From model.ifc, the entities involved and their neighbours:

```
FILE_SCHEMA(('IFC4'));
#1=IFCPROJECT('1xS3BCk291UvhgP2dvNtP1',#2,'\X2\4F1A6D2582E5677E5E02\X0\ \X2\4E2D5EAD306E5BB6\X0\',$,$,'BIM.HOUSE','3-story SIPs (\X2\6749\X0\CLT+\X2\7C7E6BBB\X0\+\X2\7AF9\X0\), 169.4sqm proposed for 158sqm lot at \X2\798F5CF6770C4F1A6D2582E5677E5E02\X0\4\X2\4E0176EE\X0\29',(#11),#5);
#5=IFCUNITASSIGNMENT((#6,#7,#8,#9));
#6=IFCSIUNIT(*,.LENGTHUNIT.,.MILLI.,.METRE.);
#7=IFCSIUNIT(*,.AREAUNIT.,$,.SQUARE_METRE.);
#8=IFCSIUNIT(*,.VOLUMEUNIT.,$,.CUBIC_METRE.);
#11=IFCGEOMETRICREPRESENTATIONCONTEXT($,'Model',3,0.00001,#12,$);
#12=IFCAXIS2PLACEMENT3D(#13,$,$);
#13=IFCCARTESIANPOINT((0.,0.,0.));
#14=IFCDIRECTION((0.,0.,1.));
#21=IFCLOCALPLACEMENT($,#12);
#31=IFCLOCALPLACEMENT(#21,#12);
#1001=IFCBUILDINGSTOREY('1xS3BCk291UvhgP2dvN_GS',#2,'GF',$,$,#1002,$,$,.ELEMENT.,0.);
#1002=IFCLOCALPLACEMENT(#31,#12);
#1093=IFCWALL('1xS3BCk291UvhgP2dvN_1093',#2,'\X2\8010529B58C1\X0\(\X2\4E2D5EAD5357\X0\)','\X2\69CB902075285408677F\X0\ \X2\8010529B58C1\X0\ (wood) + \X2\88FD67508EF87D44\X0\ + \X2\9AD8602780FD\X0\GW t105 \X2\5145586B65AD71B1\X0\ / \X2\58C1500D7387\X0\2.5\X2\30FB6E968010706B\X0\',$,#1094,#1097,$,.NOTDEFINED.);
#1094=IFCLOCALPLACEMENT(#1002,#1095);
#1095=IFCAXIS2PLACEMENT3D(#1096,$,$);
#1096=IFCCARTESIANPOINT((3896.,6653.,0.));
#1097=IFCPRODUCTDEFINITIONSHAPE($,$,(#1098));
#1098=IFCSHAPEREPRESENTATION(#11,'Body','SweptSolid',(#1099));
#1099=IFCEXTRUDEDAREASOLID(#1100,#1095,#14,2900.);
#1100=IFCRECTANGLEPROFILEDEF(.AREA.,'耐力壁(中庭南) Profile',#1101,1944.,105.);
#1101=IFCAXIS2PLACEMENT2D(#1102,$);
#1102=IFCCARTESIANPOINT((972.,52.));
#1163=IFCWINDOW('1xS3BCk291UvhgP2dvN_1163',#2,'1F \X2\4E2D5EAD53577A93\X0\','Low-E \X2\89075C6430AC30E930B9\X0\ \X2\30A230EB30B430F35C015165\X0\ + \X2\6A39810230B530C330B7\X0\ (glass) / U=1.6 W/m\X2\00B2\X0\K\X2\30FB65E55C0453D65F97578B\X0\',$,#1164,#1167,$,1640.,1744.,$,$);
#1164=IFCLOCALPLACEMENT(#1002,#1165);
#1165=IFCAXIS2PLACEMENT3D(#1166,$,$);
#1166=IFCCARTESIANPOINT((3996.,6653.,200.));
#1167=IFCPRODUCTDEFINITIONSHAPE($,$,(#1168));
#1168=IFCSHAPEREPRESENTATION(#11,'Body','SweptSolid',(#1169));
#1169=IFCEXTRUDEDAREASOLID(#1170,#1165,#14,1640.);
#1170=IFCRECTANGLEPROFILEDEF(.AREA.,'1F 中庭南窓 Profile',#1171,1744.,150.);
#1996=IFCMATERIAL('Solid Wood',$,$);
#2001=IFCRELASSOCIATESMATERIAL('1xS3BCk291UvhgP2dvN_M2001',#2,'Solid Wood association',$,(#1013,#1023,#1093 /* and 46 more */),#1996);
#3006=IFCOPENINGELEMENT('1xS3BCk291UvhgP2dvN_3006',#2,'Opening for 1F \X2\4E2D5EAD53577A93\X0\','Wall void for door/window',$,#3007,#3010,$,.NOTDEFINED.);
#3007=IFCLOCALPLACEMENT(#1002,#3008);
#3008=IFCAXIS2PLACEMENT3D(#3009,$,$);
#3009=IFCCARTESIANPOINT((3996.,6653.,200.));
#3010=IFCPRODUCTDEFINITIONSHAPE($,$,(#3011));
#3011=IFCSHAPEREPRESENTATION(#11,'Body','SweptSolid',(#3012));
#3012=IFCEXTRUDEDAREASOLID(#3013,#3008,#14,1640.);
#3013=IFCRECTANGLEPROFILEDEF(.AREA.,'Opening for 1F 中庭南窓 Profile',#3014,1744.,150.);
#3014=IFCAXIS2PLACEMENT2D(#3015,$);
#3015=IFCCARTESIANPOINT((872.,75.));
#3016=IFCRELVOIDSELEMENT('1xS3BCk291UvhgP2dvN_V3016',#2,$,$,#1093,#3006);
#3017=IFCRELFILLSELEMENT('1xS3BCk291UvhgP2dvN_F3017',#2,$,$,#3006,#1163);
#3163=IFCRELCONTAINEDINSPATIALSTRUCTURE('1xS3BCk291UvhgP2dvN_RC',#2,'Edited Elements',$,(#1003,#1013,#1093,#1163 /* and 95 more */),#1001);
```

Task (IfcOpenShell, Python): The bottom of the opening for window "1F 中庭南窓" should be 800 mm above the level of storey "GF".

```python
import numpy as np
import ifcopenshell
import ifcopenshell.api.geometry
import ifcopenshell.geom
import ifcopenshell.util.element
import ifcopenshell.util.placement
import ifcopenshell.util.shape
import ifcopenshell.util.unit

model = ifcopenshell.open("model.ifc")
unit_scale = ifcopenshell.util.unit.calculate_unit_scale(model)

window = model.by_id(1163)
opening = window.FillsVoids[0].RelatingOpeningElement
storey = ifcopenshell.util.element.get_container(window, ifc_class="IfcBuildingStorey")
level = ifcopenshell.util.placement.get_local_placement(storey.ObjectPlacement)[2, 3]

# The opening's origin need not be at the sill, so measure its lowest point.
shape = ifcopenshell.geom.create_shape(ifcopenshell.geom.settings(), opening)
bottom = ifcopenshell.util.shape.get_shape_bottom_elevation(shape, shape.geometry) / unit_scale
dz = level + 0.8 / unit_scale - bottom

shift = np.array([0.0, 0.0, dz])
# The window is not placed relative to its opening, so move both.
for product in (opening, window):
    matrix = ifcopenshell.util.placement.get_local_placement(product.ObjectPlacement)
    matrix[:3, 3] += shift
    ifcopenshell.api.geometry.edit_object_placement(model, product=product, matrix=matrix, is_si=False)

print(f"moved by {dz * unit_scale:+.3f} m")

model.write("model_updated.ifc")
```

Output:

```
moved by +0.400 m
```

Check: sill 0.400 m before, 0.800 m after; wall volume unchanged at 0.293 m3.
